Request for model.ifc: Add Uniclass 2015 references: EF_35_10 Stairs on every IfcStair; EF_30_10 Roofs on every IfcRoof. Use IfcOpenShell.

First a look at what the model holds.

```python
import ifcopenshell

model = ifcopenshell.open("model.ifc")
print(model.schema)
print("classifications:", [c.Name for c in model.by_type("IfcClassification")])
for ifc_class in ("IfcDoor", "IfcRoof", "IfcStair", "IfcWall", "IfcWindow"):
    print(ifc_class, len(model.by_type(ifc_class)))
```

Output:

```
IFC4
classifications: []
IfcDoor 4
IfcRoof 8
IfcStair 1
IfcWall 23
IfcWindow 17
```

```python
import ifcopenshell
import ifcopenshell.api.classification

model = ifcopenshell.open("model.ifc")

system = ifcopenshell.api.classification.add_classification(model, classification="Uniclass 2015")

codes = {
    "IfcStair": ("EF_35_10", "Stairs"),
    "IfcRoof": ("EF_30_10", "Roofs"),
}
for ifc_class, (code, name) in codes.items():
    products = model.by_type(ifc_class)
    ifcopenshell.api.classification.add_reference(
        model, products=products, classification=system, identification=code, name=name
    )
    print(code, len(products))

model.write("model_edited.ifc")
```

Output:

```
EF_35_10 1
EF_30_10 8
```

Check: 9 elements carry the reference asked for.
